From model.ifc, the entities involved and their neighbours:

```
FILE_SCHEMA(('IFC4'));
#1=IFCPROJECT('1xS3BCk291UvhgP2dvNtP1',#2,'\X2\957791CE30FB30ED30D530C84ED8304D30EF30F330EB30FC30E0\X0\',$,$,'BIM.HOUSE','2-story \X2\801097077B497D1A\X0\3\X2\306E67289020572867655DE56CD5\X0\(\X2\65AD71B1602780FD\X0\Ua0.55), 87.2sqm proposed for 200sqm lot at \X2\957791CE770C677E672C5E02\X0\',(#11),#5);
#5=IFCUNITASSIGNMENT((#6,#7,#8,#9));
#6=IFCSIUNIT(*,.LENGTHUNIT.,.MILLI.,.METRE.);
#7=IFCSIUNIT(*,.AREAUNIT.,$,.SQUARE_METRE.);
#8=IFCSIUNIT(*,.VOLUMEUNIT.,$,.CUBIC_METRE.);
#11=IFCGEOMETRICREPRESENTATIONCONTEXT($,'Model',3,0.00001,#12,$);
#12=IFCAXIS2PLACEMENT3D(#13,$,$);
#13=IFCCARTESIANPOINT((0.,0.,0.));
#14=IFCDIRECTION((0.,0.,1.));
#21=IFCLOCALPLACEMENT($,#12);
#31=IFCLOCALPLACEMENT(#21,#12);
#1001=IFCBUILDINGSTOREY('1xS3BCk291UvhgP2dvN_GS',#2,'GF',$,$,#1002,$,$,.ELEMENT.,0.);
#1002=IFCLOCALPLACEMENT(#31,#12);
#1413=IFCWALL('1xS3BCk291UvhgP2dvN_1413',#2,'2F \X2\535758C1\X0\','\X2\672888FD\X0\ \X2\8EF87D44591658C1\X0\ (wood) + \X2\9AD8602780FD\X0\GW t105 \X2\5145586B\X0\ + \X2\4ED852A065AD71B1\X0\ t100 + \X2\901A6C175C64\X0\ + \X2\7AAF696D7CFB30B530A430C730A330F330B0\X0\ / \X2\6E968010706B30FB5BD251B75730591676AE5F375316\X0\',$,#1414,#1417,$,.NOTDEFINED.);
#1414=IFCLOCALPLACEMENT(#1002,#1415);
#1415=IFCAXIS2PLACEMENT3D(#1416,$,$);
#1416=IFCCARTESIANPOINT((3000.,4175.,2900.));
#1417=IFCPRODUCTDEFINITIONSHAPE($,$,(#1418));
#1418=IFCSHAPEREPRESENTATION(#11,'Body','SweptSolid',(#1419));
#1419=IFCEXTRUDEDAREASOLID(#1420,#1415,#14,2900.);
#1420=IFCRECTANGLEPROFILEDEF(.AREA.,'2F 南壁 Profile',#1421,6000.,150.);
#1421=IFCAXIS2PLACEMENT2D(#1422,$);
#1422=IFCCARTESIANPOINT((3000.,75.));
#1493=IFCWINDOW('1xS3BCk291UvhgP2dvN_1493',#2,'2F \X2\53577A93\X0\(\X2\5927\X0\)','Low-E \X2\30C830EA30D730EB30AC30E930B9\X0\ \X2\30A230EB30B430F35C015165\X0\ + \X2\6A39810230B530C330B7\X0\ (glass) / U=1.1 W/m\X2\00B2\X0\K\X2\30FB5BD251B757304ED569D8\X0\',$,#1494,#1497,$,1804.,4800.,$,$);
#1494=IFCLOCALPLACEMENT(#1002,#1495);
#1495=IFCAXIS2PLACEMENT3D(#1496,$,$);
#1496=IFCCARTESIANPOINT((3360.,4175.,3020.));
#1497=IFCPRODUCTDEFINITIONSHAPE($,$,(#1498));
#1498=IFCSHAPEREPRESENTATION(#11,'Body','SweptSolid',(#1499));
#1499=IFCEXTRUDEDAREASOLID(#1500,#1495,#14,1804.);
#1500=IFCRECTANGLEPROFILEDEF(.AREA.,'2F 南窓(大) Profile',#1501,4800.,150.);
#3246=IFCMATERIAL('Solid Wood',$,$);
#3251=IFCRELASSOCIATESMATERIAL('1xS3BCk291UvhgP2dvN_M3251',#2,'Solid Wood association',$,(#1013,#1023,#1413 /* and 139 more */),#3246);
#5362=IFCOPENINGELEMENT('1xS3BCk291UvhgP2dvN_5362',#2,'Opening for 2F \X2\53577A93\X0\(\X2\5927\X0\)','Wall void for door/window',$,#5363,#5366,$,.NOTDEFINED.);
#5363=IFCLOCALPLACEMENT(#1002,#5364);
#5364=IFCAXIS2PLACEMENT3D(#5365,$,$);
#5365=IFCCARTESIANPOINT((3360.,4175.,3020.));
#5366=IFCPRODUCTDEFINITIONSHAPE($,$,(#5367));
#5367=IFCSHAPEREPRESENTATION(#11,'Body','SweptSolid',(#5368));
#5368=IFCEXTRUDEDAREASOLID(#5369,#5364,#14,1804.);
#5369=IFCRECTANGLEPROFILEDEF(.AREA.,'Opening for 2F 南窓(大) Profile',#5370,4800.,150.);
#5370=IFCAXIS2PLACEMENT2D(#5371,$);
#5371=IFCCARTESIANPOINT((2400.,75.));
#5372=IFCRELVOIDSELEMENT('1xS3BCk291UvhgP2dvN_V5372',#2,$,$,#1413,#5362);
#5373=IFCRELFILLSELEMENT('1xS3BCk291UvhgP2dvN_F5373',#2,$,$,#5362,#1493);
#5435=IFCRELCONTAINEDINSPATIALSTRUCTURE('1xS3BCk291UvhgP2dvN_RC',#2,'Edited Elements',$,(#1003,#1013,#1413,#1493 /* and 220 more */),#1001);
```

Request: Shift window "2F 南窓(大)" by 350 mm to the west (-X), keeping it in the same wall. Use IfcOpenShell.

```python
import ifcopenshell
import ifcopenshell.api.geometry
import ifcopenshell.util.placement
import ifcopenshell.util.unit

model = ifcopenshell.open("model.ifc")
unit_scale = ifcopenshell.util.unit.calculate_unit_scale(model)

window = model.by_id(1493)
opening = window.FillsVoids[0].RelatingOpeningElement
wall = opening.VoidsElements[0].RelatingBuildingElement

wall_matrix = ifcopenshell.util.placement.get_local_placement(wall.ObjectPlacement)
shift = wall_matrix[:3, 0] * -0.35 / unit_scale
before = ifcopenshell.util.placement.get_local_placement(window.ObjectPlacement)[:3, 3].copy()

# The window is not placed relative to its opening, so move both.
for product in (opening, window):
    matrix = ifcopenshell.util.placement.get_local_placement(product.ObjectPlacement)
    matrix[:3, 3] += shift
    ifcopenshell.api.geometry.edit_object_placement(model, product=product, matrix=matrix, is_si=False)

after = ifcopenshell.util.placement.get_local_placement(window.ObjectPlacement)[:3, 3]
print("window moved by", (after - before).round(3) + 0.0)

model.write("model_edited.ifc")
```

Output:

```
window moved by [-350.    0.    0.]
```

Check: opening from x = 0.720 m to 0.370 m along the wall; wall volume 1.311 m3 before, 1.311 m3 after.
